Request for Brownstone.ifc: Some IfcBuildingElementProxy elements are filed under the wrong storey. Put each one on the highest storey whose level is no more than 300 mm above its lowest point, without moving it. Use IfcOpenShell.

First a look at what the model holds.

```python
import ifcopenshell
import ifcopenshell.util.element
import ifcopenshell.util.placement

model = ifcopenshell.open("Brownstone.ifc")
print(model.schema)
for storey in model.by_type("IfcBuildingStorey"):
    level = ifcopenshell.util.placement.get_storey_elevation(storey)
    count = sum(e.is_a("IfcBuildingElementProxy") for e in ifcopenshell.util.element.get_contained(storey))
    print(storey.id(), storey.Name, round(level, 3), count, sep=" | ")
```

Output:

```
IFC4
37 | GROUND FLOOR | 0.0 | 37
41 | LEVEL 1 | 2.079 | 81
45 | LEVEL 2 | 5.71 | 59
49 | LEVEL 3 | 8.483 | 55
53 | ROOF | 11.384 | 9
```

```python
import ifcopenshell
import ifcopenshell.api.spatial
import ifcopenshell.geom
import ifcopenshell.util.element
import ifcopenshell.util.placement
import ifcopenshell.util.shape
import ifcopenshell.util.unit

model = ifcopenshell.open("Brownstone.ifc")
unit_scale = ifcopenshell.util.unit.calculate_unit_scale(model)
settings = ifcopenshell.geom.settings()

levels = sorted(
    ((ifcopenshell.util.placement.get_storey_elevation(s) * unit_scale, s) for s in model.by_type("IfcBuildingStorey")),
    key=lambda pair: pair[0],
)

for e in model.by_type("IfcBuildingElementProxy"):
    current = e.ContainedInStructure[0].RelatingStructure if e.ContainedInStructure else None
    if current is None or not current.is_a("IfcBuildingStorey"):
        continue
    shape = ifcopenshell.geom.create_shape(settings, e)
    bottom = ifcopenshell.util.shape.get_shape_bottom_elevation(shape, shape.geometry)
    below = [s for level, s in levels if level <= bottom + 0.3]
    storey = below[-1] if below else levels[0][1]
    if storey != current:
        # assign_container keeps the world position.
        ifcopenshell.api.spatial.assign_container(model, products=[e], relating_structure=storey)
        print(e.id(), current.Name, "->", storey.Name)

model.write("Brownstone-out.ifc")
```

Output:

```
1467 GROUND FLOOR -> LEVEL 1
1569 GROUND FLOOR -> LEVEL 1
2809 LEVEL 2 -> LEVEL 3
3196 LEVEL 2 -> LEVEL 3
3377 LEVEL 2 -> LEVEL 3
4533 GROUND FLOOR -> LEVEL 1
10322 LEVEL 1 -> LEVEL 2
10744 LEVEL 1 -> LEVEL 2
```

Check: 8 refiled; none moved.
